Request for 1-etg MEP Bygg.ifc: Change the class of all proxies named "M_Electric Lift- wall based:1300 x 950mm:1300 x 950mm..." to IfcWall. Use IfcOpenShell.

First a look at what the model holds.

```python
import re

import ifcopenshell

model = ifcopenshell.open("1-etg MEP Bygg.ifc")
print(model.schema)
seen = {}
for e in model.by_type("IfcBuildingElementProxy"):
    name = re.sub(r":\d+(:\d+)?$", "", e.Name or "")  # drop the element id that some exporters append
    seen[name] = seen.get(name, 0) + 1
for name, count in sorted(seen.items()):
    print(count, "x", name)
```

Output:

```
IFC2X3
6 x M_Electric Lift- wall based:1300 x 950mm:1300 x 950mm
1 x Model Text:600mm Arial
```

```python
import ifcopenshell
import ifcopenshell.api.root

model = ifcopenshell.open("1-etg MEP Bygg.ifc")

proxies = [e.id() for e in model.by_type("IfcBuildingElementProxy") if (e.Name or "").startswith("M_Electric Lift- wall based:1300 x 950mm:1300 x 950mm")]
for step_id in proxies:
    proxy = model.by_id(step_id)
    ifcopenshell.api.root.reassign_class(model, product=proxy, ifc_class="IfcWall")

print(sum(model.by_id(i).is_a("IfcWall") for i in proxies), "reclassified")

model.write("1-etg MEP Bygg-out.ifc")
```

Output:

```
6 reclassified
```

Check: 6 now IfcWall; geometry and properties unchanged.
